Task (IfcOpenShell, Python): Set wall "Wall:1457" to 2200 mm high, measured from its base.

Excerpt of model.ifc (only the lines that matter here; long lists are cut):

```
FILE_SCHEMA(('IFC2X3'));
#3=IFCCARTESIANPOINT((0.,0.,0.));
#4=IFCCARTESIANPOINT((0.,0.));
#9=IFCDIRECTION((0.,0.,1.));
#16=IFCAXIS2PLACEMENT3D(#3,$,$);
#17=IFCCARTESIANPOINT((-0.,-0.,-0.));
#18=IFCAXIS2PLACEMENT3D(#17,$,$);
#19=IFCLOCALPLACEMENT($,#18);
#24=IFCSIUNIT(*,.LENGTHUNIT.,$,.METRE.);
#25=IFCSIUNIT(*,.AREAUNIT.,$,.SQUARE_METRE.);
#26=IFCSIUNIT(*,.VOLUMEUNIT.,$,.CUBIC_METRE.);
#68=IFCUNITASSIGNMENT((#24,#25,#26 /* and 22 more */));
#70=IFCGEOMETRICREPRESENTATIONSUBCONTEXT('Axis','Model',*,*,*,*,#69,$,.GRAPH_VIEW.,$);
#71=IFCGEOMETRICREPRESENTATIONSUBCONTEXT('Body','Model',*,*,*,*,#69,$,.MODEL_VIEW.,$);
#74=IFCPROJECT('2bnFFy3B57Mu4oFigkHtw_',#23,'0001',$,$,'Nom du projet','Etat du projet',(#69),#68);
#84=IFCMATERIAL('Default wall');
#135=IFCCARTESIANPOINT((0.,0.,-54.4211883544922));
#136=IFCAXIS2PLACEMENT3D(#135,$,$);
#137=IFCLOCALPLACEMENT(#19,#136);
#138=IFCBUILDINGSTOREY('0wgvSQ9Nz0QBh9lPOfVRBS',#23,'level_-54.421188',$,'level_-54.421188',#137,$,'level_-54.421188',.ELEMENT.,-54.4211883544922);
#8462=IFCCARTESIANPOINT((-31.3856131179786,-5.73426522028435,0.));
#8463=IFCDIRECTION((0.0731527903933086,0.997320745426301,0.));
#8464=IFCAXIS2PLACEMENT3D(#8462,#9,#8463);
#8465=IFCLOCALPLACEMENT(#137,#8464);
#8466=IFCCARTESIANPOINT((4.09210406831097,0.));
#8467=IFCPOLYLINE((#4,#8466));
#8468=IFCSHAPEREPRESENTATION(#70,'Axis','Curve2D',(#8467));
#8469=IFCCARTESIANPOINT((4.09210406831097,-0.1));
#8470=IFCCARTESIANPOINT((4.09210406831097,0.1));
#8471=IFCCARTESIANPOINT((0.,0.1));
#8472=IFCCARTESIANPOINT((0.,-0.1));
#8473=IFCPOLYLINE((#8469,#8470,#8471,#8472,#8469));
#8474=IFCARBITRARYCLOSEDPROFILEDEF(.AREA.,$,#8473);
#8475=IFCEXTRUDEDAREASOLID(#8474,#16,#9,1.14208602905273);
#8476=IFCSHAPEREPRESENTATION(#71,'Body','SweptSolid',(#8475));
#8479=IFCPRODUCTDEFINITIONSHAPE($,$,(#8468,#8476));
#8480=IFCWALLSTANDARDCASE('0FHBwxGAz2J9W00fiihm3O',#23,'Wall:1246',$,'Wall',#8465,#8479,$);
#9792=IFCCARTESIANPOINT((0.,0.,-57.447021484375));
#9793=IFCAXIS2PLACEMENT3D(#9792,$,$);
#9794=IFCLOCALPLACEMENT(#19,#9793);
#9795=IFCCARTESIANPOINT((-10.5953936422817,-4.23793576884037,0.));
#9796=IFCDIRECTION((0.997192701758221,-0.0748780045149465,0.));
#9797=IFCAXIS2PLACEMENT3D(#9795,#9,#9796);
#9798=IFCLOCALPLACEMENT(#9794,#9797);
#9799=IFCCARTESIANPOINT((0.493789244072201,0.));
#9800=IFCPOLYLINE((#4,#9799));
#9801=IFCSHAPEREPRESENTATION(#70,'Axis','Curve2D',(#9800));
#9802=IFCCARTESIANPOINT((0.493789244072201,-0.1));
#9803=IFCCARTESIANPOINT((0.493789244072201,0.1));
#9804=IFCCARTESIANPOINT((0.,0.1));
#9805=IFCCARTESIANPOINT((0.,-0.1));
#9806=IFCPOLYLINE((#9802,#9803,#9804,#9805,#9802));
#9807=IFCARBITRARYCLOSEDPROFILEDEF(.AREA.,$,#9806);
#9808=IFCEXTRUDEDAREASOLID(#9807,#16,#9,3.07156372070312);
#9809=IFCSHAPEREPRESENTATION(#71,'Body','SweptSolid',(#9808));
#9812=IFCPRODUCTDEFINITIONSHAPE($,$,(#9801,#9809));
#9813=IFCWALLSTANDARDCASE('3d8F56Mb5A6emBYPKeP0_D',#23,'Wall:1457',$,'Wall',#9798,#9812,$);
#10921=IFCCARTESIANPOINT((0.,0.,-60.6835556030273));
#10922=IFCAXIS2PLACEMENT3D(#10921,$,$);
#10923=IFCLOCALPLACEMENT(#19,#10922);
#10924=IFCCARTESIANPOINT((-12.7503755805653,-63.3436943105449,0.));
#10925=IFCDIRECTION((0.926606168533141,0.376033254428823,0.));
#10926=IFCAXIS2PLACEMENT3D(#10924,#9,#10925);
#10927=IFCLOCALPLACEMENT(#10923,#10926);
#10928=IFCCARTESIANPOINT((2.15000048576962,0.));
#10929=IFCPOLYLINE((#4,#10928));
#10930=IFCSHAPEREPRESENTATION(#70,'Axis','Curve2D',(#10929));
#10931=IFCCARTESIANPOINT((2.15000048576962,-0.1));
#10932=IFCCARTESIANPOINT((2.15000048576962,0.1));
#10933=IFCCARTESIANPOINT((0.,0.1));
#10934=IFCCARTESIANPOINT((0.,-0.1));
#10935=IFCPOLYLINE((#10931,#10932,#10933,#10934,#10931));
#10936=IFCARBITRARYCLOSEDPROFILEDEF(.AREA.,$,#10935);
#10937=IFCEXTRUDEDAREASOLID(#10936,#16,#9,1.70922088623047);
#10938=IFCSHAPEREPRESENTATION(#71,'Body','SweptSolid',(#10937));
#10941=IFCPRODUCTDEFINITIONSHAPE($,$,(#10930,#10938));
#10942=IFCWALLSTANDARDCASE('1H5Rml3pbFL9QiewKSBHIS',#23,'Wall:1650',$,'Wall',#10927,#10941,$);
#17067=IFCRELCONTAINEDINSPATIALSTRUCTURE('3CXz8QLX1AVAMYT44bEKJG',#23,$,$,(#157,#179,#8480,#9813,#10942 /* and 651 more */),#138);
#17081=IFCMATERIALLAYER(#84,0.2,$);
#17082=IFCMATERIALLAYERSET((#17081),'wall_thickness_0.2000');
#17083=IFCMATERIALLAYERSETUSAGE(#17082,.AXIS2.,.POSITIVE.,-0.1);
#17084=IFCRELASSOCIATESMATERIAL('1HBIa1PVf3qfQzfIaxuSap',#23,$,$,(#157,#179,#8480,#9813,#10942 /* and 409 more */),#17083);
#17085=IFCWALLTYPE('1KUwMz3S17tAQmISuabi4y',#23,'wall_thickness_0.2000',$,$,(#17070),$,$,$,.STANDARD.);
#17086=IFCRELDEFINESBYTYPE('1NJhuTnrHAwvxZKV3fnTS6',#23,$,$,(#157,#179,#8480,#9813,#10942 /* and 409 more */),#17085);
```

```python
import ifcopenshell
import ifcopenshell.geom
import ifcopenshell.util.representation
import ifcopenshell.util.shape

model = ifcopenshell.open("model.ifc")
settings = ifcopenshell.geom.settings()


def volume(element):
    """Net volume in cubic metres, openings subtracted."""
    shape = ifcopenshell.geom.create_shape(settings, element)
    return ifcopenshell.util.shape.get_volume(shape.geometry)


wall = model.by_guid("3d8F56Mb5A6emBYPKeP0_D")
before = volume(wall)

body = ifcopenshell.util.representation.get_representation(wall, "Model", "Body")
solid = body.Items[0]
old_height = solid.Depth
solid.Depth = 2.2
after = volume(wall)

print(f"height {old_height:g} -> {solid.Depth:g}, volume {before:.3f} -> {after:.3f} m3")

model.write("model_rev.ifc")
```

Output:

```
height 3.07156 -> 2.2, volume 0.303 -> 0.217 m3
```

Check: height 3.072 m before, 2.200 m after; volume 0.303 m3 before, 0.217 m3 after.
